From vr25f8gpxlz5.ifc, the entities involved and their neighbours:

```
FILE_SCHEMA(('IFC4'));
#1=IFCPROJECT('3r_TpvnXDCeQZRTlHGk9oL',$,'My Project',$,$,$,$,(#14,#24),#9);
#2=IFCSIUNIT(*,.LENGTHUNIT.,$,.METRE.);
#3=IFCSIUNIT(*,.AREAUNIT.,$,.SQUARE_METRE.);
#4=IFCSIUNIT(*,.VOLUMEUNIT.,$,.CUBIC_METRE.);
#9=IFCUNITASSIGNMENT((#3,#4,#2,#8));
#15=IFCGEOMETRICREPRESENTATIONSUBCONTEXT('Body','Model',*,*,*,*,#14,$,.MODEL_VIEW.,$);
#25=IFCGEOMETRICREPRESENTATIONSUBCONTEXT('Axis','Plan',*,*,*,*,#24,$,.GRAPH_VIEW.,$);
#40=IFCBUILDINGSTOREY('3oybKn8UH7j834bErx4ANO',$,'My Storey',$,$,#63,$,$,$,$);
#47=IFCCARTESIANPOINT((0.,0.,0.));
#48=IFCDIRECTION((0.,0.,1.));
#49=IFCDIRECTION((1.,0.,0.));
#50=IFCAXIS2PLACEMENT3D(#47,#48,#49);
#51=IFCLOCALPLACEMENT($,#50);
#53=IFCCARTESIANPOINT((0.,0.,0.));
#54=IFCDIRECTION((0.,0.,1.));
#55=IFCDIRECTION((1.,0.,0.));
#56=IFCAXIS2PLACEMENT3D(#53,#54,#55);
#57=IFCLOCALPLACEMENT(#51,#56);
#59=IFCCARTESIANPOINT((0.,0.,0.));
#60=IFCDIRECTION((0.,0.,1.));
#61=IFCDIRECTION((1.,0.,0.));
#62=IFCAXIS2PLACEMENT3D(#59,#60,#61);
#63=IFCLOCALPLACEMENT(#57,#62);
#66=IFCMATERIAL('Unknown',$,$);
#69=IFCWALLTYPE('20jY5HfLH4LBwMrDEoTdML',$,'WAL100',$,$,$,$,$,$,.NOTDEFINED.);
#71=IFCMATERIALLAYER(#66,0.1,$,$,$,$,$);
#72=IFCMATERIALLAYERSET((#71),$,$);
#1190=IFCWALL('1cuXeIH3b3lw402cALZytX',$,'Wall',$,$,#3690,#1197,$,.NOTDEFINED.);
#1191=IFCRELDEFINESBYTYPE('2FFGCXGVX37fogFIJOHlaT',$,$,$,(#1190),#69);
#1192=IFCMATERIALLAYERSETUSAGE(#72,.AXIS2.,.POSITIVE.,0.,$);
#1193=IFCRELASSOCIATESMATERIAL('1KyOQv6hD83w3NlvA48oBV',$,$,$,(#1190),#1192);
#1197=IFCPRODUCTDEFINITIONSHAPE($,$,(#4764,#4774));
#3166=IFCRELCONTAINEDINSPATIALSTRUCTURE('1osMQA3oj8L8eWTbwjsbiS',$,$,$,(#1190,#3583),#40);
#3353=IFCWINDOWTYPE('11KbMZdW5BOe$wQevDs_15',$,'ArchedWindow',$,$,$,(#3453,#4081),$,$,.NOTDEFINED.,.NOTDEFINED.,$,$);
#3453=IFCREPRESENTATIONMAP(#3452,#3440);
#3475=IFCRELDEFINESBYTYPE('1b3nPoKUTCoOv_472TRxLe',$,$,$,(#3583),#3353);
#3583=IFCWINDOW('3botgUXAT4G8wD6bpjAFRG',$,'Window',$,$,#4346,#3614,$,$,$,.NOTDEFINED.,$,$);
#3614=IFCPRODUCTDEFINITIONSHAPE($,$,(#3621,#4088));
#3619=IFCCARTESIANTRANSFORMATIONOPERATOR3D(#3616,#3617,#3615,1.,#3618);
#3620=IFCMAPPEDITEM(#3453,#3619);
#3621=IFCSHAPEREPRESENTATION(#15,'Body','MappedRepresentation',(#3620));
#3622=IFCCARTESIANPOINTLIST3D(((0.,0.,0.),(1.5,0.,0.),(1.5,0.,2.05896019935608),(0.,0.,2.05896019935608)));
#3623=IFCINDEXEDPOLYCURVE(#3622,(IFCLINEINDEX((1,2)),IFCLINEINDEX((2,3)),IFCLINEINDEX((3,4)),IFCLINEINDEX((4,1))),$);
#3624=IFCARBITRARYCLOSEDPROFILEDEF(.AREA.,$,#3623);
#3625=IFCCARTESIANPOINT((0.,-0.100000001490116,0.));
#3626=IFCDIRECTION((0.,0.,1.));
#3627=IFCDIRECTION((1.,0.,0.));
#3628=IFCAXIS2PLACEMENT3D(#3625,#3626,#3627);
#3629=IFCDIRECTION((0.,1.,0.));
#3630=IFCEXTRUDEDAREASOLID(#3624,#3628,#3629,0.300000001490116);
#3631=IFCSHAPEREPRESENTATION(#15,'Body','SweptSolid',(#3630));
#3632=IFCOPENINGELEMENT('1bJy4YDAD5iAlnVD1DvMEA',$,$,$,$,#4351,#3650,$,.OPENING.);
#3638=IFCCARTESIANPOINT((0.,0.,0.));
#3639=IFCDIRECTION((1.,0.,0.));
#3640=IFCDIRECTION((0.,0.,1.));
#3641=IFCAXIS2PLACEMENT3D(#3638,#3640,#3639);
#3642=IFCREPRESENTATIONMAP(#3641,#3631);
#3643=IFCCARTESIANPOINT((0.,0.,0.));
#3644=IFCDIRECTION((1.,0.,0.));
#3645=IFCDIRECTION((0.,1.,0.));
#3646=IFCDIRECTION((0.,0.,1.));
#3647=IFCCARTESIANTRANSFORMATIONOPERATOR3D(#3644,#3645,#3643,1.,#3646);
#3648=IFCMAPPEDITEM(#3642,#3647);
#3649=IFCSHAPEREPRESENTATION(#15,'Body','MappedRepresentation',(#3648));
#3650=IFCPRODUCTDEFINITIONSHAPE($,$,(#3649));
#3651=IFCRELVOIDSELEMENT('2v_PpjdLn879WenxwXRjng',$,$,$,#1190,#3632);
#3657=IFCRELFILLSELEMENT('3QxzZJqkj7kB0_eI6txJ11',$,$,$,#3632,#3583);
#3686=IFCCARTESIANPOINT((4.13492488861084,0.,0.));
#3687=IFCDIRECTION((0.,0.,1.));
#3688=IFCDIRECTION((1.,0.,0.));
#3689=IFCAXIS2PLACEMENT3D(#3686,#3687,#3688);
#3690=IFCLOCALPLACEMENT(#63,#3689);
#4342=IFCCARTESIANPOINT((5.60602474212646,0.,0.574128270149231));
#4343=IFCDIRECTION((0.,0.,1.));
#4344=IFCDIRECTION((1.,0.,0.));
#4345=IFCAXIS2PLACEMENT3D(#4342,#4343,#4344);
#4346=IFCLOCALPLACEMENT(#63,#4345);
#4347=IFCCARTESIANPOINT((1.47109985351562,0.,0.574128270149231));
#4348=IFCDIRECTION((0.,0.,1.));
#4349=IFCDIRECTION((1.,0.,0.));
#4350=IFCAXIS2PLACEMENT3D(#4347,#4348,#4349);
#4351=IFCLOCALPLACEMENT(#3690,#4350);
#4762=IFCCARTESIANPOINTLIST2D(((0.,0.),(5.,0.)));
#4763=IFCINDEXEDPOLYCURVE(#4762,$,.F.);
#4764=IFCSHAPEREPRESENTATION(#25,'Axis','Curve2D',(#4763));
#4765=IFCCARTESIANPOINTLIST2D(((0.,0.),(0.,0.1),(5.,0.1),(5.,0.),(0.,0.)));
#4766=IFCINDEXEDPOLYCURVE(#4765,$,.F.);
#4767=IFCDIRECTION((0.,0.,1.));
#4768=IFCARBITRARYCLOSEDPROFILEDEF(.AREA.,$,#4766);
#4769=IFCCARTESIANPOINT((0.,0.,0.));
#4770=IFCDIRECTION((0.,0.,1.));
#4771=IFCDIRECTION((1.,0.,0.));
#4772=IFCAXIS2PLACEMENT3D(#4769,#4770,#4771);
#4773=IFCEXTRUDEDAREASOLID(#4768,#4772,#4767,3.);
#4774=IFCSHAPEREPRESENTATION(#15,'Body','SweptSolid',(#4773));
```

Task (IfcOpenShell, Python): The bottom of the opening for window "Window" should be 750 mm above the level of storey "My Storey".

```python
import numpy as np
import ifcopenshell
import ifcopenshell.api.geometry
import ifcopenshell.geom
import ifcopenshell.util.element
import ifcopenshell.util.placement
import ifcopenshell.util.shape
import ifcopenshell.util.unit

model = ifcopenshell.open("vr25f8gpxlz5.ifc")
unit_scale = ifcopenshell.util.unit.calculate_unit_scale(model)

window = model.by_guid("3botgUXAT4G8wD6bpjAFRG")
opening = window.FillsVoids[0].RelatingOpeningElement
storey = ifcopenshell.util.element.get_container(window, ifc_class="IfcBuildingStorey")
level = ifcopenshell.util.placement.get_local_placement(storey.ObjectPlacement)[2, 3]

# The opening's origin need not be at the sill, so measure its lowest point.
shape = ifcopenshell.geom.create_shape(ifcopenshell.geom.settings(), opening)
bottom = ifcopenshell.util.shape.get_shape_bottom_elevation(shape, shape.geometry) / unit_scale
dz = level + 0.75 - bottom

shift = np.array([0.0, 0.0, dz])
# The window is not placed relative to its opening, so move both.
for product in (opening, window):
    matrix = ifcopenshell.util.placement.get_local_placement(product.ObjectPlacement)
    matrix[:3, 3] += shift
    ifcopenshell.api.geometry.edit_object_placement(model, product=product, matrix=matrix, is_si=False)

print(f"moved by {dz * unit_scale:+.3f} m")

model.write("vr25f8gpxlz5_rev.ifc")
```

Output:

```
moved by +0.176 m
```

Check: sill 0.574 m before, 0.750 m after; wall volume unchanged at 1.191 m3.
